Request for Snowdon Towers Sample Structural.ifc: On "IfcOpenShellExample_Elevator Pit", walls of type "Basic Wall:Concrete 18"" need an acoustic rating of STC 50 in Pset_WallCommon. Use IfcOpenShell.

First a look at what the model holds.

```python
import ifcopenshell
import ifcopenshell.util.element

model = ifcopenshell.open("Snowdon Towers Sample Structural.ifc")
print(model.schema)
storey = next(s for s in model.by_type("IfcBuildingStorey") if s.Name == "IfcOpenShellExample_Elevator Pit")
walls = [e for e in ifcopenshell.util.element.get_decomposition(storey) if e.is_a("IfcWall")]
seen = {}
for e in walls:
    element_type = ifcopenshell.util.element.get_type(e)
    key = (element_type.Name if element_type != e and element_type else None, ifcopenshell.util.element.get_pset(e, "Pset_WallCommon", "AcousticRating"))
    seen[key] = seen.get(key, 0) + 1
for (name, value), count in sorted(seen.items(), key=str):
    print(count, "x", name, "|", value)
```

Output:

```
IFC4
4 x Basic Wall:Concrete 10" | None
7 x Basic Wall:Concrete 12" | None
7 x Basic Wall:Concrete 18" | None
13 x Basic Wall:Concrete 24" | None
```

```python
import ifcopenshell
import ifcopenshell.api.pset
import ifcopenshell.util.element

model = ifcopenshell.open("Snowdon Towers Sample Structural.ifc")

storey = next(s for s in model.by_type("IfcBuildingStorey") if s.Name == "IfcOpenShellExample_Elevator Pit")
walls = [e for e in ifcopenshell.util.element.get_decomposition(storey) if e.is_a("IfcWall")]

count = 0
for e in walls:
    element_type = ifcopenshell.util.element.get_type(e)
    if element_type in (None, e) or element_type.Name != 'Basic Wall:Concrete 18"':
        continue
    # add_pset returns the element's existing set when there is one.
    pset = ifcopenshell.api.pset.add_pset(model, product=e, name="Pset_WallCommon")
    ifcopenshell.api.pset.edit_pset(model, pset=pset, properties={"AcousticRating": "STC 50"})
    count += 1

print(count, "walls updated")

model.write("Snowdon Towers Sample Structural_rev.ifc")
```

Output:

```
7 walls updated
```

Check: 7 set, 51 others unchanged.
